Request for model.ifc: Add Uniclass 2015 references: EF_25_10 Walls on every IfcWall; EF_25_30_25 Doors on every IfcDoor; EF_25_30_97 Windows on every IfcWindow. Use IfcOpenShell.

First a look at what the model holds.

```python
import ifcopenshell

model = ifcopenshell.open("model.ifc")
print(model.schema)
print("classifications:", [c.Name for c in model.by_type("IfcClassification")])
for ifc_class in ("IfcDoor", "IfcRoof", "IfcStair", "IfcWall", "IfcWindow"):
    print(ifc_class, len(model.by_type(ifc_class)))
```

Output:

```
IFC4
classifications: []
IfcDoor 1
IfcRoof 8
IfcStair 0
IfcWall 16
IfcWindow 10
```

```python
import ifcopenshell
import ifcopenshell.api.classification

model = ifcopenshell.open("model.ifc")

system = ifcopenshell.api.classification.add_classification(model, classification="Uniclass 2015")

codes = {
    "IfcWall": ("EF_25_10", "Walls"),
    "IfcDoor": ("EF_25_30_25", "Doors"),
    "IfcWindow": ("EF_25_30_97", "Windows"),
}
for ifc_class, (code, name) in codes.items():
    products = model.by_type(ifc_class)
    ifcopenshell.api.classification.add_reference(
        model, products=products, classification=system, identification=code, name=name
    )
    print(code, len(products))

model.write("model_v2.ifc")
```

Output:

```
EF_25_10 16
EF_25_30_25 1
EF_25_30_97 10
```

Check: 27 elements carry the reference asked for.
